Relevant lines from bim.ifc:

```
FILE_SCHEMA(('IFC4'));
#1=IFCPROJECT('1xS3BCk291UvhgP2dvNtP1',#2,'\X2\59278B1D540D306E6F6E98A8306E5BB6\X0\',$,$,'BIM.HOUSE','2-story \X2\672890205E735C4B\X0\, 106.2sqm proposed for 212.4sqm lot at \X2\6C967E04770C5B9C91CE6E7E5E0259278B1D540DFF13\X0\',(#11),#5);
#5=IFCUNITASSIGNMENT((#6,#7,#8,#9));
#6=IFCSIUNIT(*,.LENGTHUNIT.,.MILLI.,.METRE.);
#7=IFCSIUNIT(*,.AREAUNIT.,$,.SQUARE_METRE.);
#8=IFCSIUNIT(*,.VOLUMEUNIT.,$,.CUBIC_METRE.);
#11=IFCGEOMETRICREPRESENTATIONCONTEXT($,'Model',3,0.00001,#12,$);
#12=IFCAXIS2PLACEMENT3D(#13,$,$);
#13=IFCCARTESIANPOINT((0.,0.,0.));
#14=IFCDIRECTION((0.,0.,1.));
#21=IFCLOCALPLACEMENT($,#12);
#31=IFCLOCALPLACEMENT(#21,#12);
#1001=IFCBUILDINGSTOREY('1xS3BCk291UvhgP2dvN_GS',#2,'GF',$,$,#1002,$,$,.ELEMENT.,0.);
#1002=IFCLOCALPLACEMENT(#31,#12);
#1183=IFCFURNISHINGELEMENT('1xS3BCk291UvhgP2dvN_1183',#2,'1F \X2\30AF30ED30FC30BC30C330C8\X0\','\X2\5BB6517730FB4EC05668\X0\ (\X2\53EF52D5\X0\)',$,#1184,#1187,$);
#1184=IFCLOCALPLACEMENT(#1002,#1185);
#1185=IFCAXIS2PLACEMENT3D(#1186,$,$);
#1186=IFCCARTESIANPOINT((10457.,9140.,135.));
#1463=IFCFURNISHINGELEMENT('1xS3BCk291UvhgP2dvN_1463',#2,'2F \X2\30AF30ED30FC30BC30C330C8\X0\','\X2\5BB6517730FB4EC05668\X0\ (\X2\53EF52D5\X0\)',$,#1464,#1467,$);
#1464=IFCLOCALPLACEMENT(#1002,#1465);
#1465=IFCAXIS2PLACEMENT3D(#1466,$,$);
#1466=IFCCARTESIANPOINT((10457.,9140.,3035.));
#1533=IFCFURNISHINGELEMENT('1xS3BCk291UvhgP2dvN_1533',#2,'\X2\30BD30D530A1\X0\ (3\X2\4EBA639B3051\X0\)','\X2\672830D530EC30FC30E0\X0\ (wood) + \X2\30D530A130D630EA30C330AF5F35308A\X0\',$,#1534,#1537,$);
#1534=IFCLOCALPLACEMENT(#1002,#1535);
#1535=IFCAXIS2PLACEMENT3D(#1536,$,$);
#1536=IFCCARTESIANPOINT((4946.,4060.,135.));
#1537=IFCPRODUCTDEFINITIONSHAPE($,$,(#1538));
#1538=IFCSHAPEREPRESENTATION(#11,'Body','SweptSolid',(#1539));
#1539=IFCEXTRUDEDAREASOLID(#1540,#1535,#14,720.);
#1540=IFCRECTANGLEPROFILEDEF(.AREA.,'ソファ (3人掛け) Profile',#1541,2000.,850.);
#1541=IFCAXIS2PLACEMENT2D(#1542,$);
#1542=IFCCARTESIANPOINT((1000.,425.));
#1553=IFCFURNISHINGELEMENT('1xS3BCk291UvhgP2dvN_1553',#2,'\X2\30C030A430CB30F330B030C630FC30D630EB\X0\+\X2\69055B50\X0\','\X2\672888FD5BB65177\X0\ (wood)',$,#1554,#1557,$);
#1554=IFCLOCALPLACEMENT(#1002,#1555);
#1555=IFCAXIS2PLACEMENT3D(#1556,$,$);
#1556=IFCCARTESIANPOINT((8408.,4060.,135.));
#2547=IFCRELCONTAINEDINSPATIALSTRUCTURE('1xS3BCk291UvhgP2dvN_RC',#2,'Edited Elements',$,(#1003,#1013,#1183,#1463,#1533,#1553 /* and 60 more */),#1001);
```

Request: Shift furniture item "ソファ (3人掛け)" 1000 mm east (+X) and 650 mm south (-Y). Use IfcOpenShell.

```python
import ifcopenshell
import ifcopenshell.api.geometry
import ifcopenshell.util.placement
import ifcopenshell.util.unit

model = ifcopenshell.open("bim.ifc")
unit_scale = ifcopenshell.util.unit.calculate_unit_scale(model)

item = model.by_id(1533)
matrix = ifcopenshell.util.placement.get_local_placement(item.ObjectPlacement)
matrix[0, 3] += 1 / unit_scale
matrix[1, 3] -= 0.65 / unit_scale
ifcopenshell.api.geometry.edit_object_placement(model, product=item, matrix=matrix, is_si=False)

print(ifcopenshell.util.placement.get_local_placement(item.ObjectPlacement).round(3) + 0.0)

model.write("bim-out.ifc")
```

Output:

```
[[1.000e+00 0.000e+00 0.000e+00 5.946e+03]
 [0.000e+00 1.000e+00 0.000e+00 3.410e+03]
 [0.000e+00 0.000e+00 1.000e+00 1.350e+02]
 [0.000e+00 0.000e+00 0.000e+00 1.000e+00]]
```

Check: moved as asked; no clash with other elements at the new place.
